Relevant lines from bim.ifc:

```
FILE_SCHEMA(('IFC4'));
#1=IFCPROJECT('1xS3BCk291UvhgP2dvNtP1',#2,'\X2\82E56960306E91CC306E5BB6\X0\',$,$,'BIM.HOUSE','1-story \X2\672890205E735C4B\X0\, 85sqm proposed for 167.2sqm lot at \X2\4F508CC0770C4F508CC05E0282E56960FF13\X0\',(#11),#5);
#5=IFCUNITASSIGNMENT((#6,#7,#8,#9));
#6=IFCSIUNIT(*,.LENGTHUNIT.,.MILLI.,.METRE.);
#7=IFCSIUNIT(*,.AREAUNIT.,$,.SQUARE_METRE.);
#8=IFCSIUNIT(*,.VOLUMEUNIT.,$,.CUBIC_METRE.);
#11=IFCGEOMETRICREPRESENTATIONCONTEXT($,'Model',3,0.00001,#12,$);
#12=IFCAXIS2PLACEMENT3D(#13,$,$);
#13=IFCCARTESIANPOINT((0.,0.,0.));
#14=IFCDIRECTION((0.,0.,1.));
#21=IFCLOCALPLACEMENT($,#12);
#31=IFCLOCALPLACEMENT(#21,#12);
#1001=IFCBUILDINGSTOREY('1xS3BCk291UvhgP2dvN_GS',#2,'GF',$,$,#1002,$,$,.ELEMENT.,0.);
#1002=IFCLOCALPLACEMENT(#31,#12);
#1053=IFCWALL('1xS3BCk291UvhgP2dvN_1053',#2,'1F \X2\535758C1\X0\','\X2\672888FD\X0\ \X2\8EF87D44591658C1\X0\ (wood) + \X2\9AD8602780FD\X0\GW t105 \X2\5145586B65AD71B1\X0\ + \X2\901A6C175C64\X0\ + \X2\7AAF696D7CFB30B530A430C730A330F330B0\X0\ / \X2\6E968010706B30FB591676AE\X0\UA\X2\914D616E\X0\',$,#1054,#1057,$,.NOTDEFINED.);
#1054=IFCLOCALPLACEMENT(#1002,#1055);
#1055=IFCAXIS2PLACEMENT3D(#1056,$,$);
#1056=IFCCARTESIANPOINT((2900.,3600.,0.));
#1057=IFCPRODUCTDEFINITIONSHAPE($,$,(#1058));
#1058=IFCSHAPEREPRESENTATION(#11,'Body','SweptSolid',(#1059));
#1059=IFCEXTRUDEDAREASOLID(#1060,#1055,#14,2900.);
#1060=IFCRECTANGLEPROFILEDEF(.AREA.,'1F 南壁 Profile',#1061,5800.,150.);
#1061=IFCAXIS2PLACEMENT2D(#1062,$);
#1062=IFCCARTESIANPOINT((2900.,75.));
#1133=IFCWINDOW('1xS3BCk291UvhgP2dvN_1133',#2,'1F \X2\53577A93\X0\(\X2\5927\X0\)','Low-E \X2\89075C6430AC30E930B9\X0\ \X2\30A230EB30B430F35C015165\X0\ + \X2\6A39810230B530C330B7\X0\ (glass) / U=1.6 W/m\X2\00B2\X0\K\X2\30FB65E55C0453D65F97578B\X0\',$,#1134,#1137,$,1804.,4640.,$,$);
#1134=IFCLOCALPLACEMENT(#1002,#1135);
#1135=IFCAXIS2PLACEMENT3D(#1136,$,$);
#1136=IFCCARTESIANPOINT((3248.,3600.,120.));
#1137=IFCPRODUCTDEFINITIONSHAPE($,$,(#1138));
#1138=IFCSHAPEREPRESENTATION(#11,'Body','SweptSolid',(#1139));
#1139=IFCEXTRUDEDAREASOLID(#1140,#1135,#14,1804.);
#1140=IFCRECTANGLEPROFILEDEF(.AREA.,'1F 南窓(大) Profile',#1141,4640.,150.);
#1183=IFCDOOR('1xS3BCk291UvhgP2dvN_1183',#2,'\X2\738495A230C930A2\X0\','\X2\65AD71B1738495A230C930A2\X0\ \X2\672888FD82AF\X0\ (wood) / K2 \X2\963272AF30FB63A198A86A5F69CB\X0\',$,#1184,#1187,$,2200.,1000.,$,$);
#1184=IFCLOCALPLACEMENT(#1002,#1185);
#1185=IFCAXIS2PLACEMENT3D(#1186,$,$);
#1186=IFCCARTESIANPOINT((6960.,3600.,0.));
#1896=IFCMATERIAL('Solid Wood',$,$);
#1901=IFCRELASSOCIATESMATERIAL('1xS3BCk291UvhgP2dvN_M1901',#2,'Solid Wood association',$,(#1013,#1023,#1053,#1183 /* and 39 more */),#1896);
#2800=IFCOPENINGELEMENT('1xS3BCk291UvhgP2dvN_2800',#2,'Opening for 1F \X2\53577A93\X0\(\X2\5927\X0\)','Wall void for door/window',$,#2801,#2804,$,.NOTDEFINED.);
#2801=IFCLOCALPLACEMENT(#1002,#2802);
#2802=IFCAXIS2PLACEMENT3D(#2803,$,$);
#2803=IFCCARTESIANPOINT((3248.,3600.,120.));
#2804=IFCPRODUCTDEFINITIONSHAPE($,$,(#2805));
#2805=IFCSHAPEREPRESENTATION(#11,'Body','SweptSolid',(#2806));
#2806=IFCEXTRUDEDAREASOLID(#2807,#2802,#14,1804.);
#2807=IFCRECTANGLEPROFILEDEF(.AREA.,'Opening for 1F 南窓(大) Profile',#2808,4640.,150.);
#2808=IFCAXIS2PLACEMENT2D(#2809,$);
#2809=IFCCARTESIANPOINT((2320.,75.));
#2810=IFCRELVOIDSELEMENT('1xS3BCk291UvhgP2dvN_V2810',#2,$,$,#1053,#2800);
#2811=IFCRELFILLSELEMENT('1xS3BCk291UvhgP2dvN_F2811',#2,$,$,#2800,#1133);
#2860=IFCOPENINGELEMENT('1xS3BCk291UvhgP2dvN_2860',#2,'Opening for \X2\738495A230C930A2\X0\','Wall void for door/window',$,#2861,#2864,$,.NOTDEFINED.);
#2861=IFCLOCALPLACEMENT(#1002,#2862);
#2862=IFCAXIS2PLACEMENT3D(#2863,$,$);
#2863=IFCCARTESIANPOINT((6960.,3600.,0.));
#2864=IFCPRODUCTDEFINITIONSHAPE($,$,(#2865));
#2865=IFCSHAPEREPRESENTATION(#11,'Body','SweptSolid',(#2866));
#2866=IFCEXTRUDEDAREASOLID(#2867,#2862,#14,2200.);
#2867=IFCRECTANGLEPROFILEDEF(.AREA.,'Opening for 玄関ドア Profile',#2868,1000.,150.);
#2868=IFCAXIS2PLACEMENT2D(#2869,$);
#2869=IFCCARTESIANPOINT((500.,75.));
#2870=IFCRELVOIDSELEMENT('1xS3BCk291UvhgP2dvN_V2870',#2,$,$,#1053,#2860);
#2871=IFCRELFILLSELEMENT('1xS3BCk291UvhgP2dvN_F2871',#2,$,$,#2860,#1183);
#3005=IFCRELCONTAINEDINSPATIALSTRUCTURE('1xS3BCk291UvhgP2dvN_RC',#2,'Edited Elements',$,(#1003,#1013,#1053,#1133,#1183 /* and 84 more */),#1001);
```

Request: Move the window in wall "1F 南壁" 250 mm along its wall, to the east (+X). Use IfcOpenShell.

```python
import ifcopenshell
import ifcopenshell.api.geometry
import ifcopenshell.util.placement

model = ifcopenshell.open("bim.ifc")

window = model.by_guid("1xS3BCk291UvhgP2dvN_1133")
opening = window.FillsVoids[0].RelatingOpeningElement
wall = opening.VoidsElements[0].RelatingBuildingElement

wall_matrix = ifcopenshell.util.placement.get_local_placement(wall.ObjectPlacement)
shift = wall_matrix[:3, 0] * 250.0
before = ifcopenshell.util.placement.get_local_placement(window.ObjectPlacement)[:3, 3].copy()

# The window is not placed relative to its opening, so move both.
for product in (opening, window):
    matrix = ifcopenshell.util.placement.get_local_placement(product.ObjectPlacement)
    matrix[:3, 3] += shift
    ifcopenshell.api.geometry.edit_object_placement(model, product=product, matrix=matrix, is_si=False)

after = ifcopenshell.util.placement.get_local_placement(window.ObjectPlacement)[:3, 3]
print("window moved by", (after - before).round(3) + 0.0)

model.write("bim_edited.ifc")
```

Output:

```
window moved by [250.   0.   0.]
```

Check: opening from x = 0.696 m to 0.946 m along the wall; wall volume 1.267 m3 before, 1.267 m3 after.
